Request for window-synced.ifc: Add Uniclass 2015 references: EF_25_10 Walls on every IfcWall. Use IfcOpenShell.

First a look at what the model holds.

```python
import ifcopenshell

model = ifcopenshell.open("window-synced.ifc")
print(model.schema)
print("classifications:", [c.Name for c in model.by_type("IfcClassification")])
for ifc_class in ("IfcDoor", "IfcRoof", "IfcStair", "IfcWall", "IfcWindow"):
    print(ifc_class, len(model.by_type(ifc_class)))
```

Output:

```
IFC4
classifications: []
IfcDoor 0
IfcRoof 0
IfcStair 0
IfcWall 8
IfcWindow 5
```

```python
import ifcopenshell
import ifcopenshell.api.classification

model = ifcopenshell.open("window-synced.ifc")

system = ifcopenshell.api.classification.add_classification(model, classification="Uniclass 2015")

codes = {
    "IfcWall": ("EF_25_10", "Walls"),
}
for ifc_class, (code, name) in codes.items():
    products = model.by_type(ifc_class)
    ifcopenshell.api.classification.add_reference(
        model, products=products, classification=system, identification=code, name=name
    )
    print(code, len(products))

model.write("window-synced_edited.ifc")
```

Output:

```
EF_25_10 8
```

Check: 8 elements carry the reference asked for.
